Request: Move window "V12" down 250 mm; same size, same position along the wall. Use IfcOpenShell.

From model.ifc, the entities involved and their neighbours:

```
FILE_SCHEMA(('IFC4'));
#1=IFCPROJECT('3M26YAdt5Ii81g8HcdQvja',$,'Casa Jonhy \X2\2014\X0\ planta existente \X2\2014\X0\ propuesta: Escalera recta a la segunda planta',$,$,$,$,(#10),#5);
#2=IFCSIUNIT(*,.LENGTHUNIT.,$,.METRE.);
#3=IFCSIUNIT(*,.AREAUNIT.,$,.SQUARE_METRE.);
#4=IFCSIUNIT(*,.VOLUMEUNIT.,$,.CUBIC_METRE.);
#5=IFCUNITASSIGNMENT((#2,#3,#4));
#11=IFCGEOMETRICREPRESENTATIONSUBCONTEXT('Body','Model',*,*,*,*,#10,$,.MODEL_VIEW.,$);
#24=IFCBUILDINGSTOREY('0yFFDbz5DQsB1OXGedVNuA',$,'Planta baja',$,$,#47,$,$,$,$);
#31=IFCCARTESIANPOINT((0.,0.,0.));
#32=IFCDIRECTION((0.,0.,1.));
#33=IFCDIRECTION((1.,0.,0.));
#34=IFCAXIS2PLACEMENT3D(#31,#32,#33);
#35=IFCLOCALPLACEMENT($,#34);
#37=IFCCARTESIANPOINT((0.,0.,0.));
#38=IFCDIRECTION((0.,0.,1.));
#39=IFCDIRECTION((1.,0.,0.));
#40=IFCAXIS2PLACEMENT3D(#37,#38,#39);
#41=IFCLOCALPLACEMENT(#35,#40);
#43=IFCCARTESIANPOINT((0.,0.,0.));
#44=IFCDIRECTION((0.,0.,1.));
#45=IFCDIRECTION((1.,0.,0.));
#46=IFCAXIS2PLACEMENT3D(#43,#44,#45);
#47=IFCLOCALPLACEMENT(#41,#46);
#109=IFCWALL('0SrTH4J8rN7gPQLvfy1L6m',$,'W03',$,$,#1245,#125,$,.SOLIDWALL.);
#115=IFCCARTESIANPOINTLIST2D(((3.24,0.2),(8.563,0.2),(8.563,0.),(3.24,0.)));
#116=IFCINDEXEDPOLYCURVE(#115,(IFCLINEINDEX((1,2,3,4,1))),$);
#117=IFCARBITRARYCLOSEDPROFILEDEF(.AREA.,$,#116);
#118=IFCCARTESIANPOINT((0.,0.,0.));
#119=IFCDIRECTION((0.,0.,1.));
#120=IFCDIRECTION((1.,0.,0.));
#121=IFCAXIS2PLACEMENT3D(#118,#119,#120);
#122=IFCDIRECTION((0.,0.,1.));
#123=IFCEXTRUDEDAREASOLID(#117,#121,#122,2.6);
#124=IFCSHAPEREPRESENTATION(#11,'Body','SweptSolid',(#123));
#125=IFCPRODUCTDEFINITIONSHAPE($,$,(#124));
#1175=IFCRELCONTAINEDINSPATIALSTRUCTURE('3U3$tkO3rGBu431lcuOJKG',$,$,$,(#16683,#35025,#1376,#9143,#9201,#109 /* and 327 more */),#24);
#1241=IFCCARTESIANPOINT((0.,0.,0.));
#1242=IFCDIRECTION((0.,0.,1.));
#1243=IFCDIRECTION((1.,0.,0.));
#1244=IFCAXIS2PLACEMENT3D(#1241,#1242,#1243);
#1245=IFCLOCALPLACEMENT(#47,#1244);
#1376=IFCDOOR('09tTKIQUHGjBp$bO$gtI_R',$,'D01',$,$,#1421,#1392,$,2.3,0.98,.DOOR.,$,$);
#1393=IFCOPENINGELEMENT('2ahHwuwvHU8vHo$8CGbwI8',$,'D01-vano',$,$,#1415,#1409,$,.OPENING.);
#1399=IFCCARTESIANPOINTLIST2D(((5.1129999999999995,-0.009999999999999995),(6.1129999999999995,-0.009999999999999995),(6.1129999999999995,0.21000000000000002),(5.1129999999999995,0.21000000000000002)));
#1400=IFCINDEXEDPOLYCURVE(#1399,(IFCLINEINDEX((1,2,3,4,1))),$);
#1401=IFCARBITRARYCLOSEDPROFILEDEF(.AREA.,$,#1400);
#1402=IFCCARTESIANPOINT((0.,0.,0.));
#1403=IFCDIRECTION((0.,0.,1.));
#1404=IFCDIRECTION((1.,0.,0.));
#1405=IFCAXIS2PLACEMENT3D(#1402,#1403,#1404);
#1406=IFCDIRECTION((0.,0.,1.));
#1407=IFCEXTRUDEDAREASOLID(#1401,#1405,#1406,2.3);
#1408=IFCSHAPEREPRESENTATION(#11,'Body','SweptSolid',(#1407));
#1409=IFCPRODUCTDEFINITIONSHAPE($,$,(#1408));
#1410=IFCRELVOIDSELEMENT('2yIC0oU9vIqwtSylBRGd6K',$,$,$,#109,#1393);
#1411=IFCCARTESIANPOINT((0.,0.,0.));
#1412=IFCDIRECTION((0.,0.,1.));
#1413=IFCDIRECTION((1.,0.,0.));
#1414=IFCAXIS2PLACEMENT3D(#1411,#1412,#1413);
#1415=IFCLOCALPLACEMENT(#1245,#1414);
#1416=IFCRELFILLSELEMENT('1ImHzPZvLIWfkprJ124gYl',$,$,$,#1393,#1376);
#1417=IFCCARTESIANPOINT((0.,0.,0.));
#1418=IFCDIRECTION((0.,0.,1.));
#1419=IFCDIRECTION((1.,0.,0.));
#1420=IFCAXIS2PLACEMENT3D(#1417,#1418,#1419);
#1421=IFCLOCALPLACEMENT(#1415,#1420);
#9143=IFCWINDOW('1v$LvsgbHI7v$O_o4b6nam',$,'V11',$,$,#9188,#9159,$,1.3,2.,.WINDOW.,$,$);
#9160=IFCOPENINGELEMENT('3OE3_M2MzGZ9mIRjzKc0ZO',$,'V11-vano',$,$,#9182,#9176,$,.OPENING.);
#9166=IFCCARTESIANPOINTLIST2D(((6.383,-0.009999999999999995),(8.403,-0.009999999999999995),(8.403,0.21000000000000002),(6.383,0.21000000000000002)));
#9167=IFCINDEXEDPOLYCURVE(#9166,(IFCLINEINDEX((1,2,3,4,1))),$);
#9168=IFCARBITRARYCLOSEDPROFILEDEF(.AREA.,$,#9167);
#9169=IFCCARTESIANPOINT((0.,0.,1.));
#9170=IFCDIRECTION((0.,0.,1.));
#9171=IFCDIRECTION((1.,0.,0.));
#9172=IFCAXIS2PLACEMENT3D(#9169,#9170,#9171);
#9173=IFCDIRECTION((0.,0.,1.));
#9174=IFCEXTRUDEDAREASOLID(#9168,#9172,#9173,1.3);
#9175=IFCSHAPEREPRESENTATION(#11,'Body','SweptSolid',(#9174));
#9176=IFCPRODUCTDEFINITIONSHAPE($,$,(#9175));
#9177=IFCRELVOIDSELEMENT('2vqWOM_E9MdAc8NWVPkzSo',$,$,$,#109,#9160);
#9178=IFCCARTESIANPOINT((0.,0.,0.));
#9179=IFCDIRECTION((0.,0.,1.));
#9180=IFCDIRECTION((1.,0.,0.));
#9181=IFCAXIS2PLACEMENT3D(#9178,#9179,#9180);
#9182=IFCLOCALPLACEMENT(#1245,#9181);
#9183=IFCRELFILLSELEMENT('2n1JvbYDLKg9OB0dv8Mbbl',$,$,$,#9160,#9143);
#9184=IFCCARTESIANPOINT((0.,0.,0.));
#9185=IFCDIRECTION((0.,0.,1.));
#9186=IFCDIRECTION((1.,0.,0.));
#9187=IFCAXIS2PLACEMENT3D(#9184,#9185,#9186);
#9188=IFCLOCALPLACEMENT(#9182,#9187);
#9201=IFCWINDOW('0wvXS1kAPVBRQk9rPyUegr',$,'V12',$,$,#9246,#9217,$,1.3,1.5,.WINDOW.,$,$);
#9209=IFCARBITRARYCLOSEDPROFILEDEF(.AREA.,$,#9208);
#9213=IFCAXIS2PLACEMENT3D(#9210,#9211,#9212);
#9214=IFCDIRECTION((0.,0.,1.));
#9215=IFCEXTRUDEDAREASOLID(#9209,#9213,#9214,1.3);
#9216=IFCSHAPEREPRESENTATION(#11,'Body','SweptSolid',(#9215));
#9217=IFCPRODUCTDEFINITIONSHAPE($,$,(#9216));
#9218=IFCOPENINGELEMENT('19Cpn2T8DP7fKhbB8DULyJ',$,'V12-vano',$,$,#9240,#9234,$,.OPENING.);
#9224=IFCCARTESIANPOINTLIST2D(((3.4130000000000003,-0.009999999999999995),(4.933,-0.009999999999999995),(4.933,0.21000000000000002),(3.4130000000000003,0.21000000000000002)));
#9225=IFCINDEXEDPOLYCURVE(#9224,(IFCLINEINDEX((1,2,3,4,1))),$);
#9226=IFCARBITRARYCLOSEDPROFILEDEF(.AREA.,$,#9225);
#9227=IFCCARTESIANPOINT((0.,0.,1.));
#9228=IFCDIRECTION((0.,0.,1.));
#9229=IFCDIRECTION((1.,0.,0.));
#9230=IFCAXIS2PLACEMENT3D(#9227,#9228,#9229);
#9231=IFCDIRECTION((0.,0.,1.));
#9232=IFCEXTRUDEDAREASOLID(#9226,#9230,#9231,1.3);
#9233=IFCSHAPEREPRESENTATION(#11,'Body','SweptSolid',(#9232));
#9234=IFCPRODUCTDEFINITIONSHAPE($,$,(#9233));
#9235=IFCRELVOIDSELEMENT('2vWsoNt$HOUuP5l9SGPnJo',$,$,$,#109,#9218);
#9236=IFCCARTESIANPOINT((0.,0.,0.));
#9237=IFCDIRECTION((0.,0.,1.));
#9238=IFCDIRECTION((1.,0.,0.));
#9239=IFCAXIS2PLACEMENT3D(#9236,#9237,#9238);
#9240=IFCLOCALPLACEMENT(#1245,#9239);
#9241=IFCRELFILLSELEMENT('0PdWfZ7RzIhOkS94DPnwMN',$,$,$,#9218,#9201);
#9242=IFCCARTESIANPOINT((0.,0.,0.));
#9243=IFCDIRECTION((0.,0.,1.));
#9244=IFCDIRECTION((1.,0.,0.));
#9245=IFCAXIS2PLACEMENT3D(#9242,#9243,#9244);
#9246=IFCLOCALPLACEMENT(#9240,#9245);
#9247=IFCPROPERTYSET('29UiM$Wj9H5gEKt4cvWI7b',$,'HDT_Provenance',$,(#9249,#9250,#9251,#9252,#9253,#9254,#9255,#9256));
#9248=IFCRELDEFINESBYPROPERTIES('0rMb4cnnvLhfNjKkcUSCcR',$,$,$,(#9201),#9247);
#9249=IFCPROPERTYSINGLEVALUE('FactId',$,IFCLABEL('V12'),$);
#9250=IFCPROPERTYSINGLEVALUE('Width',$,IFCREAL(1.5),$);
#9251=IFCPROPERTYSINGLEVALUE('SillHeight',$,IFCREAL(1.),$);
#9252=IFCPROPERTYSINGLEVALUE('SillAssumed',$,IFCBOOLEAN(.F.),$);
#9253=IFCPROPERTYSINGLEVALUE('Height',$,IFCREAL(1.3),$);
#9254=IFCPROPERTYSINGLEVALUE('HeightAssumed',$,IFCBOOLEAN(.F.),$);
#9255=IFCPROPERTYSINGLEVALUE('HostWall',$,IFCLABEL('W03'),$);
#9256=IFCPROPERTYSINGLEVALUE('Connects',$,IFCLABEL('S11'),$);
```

```python
import numpy as np
import ifcopenshell
import ifcopenshell.api.geometry
import ifcopenshell.api.pset
import ifcopenshell.util.element
import ifcopenshell.util.placement
import ifcopenshell.util.unit

model = ifcopenshell.open("model.ifc")
unit_scale = ifcopenshell.util.unit.calculate_unit_scale(model)

window = model.by_guid("0wvXS1kAPVBRQk9rPyUegr")
opening = window.FillsVoids[0].RelatingOpeningElement
dz = -0.25

shift = np.array([0.0, 0.0, dz])
# The window is placed relative to its opening, so it follows when the opening moves.
matrix = ifcopenshell.util.placement.get_local_placement(opening.ObjectPlacement)
matrix[:3, 3] += shift
ifcopenshell.api.geometry.edit_object_placement(
    model, product=opening, matrix=matrix, is_si=False, should_transform_children=True
)

# Keep the stored heights in step.
pset = model.by_id(ifcopenshell.util.element.get_pset(window, "HDT_Provenance", should_inherit=False)["id"])
ifcopenshell.api.pset.edit_pset(model, pset=pset, properties={
    "SillHeight": model.create_entity("IfcReal", ifcopenshell.util.element.get_pset(window, "HDT_Provenance", "SillHeight") + dz),
})

print(f"moved by {dz * unit_scale:+.3f} m")

model.write("model_updated.ifc")
```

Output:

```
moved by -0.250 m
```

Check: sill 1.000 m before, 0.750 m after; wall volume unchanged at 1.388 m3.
